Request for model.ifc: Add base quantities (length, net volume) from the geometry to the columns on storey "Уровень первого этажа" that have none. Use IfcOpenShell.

First a look at what the model holds.

```python
import ifcopenshell
import ifcopenshell.util.element
import ifcopenshell.util.unit

model = ifcopenshell.open("model.ifc")
print(model.schema)
for unit_type in ("LENGTHUNIT", "AREAUNIT", "VOLUMEUNIT"):
    print(unit_type, ifcopenshell.util.unit.calculate_unit_scale(model, unit_type))
storey = next(s for s in model.by_type("IfcBuildingStorey") if s.Name == "Уровень первого этажа")
columns = [e for e in ifcopenshell.util.element.get_decomposition(storey) if e.is_a("IfcColumn")]
for e in sorted(columns, key=lambda e: e.id()):
    print(e.id(), e.is_a(), e.Name, list(ifcopenshell.util.element.get_psets(e, qtos_only=True)), sep=" | ")
```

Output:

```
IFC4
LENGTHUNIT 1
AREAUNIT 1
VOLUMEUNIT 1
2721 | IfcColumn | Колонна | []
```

```python
import ifcopenshell
import ifcopenshell.api.pset
import ifcopenshell.geom
import ifcopenshell.util.element
import ifcopenshell.util.shape
import ifcopenshell.util.unit

model = ifcopenshell.open("model.ifc")
unit_scale = ifcopenshell.util.unit.calculate_unit_scale(model)
volume_scale = ifcopenshell.util.unit.calculate_unit_scale(model, "VOLUMEUNIT")
settings = ifcopenshell.geom.settings()

storey = next(s for s in model.by_type("IfcBuildingStorey") if s.Name == "Уровень первого этажа")
columns = [e for e in ifcopenshell.util.element.get_decomposition(storey) if e.is_a("IfcColumn")]

for e in sorted(columns, key=lambda e: e.id()):
    if ifcopenshell.util.element.get_psets(e, qtos_only=True, should_inherit=False):
        continue
    # Geometry comes back in metres, in the element's own axes.
    shape = ifcopenshell.geom.create_shape(settings, e)
    values = {
        "Length": ifcopenshell.util.shape.get_z(shape.geometry) / unit_scale,
        "NetVolume": ifcopenshell.util.shape.get_volume(shape.geometry) / volume_scale,
    }
    qto = ifcopenshell.api.pset.add_qto(model, product=e, name="Qto_ColumnBaseQuantities")
    ifcopenshell.api.pset.edit_qto(model, qto=qto, properties=values)
    print(e.id(), {k: round(v, 3) for k, v in values.items()})

model.write("model_updated.ifc")
```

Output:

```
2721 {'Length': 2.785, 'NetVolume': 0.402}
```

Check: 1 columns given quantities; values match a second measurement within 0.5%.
